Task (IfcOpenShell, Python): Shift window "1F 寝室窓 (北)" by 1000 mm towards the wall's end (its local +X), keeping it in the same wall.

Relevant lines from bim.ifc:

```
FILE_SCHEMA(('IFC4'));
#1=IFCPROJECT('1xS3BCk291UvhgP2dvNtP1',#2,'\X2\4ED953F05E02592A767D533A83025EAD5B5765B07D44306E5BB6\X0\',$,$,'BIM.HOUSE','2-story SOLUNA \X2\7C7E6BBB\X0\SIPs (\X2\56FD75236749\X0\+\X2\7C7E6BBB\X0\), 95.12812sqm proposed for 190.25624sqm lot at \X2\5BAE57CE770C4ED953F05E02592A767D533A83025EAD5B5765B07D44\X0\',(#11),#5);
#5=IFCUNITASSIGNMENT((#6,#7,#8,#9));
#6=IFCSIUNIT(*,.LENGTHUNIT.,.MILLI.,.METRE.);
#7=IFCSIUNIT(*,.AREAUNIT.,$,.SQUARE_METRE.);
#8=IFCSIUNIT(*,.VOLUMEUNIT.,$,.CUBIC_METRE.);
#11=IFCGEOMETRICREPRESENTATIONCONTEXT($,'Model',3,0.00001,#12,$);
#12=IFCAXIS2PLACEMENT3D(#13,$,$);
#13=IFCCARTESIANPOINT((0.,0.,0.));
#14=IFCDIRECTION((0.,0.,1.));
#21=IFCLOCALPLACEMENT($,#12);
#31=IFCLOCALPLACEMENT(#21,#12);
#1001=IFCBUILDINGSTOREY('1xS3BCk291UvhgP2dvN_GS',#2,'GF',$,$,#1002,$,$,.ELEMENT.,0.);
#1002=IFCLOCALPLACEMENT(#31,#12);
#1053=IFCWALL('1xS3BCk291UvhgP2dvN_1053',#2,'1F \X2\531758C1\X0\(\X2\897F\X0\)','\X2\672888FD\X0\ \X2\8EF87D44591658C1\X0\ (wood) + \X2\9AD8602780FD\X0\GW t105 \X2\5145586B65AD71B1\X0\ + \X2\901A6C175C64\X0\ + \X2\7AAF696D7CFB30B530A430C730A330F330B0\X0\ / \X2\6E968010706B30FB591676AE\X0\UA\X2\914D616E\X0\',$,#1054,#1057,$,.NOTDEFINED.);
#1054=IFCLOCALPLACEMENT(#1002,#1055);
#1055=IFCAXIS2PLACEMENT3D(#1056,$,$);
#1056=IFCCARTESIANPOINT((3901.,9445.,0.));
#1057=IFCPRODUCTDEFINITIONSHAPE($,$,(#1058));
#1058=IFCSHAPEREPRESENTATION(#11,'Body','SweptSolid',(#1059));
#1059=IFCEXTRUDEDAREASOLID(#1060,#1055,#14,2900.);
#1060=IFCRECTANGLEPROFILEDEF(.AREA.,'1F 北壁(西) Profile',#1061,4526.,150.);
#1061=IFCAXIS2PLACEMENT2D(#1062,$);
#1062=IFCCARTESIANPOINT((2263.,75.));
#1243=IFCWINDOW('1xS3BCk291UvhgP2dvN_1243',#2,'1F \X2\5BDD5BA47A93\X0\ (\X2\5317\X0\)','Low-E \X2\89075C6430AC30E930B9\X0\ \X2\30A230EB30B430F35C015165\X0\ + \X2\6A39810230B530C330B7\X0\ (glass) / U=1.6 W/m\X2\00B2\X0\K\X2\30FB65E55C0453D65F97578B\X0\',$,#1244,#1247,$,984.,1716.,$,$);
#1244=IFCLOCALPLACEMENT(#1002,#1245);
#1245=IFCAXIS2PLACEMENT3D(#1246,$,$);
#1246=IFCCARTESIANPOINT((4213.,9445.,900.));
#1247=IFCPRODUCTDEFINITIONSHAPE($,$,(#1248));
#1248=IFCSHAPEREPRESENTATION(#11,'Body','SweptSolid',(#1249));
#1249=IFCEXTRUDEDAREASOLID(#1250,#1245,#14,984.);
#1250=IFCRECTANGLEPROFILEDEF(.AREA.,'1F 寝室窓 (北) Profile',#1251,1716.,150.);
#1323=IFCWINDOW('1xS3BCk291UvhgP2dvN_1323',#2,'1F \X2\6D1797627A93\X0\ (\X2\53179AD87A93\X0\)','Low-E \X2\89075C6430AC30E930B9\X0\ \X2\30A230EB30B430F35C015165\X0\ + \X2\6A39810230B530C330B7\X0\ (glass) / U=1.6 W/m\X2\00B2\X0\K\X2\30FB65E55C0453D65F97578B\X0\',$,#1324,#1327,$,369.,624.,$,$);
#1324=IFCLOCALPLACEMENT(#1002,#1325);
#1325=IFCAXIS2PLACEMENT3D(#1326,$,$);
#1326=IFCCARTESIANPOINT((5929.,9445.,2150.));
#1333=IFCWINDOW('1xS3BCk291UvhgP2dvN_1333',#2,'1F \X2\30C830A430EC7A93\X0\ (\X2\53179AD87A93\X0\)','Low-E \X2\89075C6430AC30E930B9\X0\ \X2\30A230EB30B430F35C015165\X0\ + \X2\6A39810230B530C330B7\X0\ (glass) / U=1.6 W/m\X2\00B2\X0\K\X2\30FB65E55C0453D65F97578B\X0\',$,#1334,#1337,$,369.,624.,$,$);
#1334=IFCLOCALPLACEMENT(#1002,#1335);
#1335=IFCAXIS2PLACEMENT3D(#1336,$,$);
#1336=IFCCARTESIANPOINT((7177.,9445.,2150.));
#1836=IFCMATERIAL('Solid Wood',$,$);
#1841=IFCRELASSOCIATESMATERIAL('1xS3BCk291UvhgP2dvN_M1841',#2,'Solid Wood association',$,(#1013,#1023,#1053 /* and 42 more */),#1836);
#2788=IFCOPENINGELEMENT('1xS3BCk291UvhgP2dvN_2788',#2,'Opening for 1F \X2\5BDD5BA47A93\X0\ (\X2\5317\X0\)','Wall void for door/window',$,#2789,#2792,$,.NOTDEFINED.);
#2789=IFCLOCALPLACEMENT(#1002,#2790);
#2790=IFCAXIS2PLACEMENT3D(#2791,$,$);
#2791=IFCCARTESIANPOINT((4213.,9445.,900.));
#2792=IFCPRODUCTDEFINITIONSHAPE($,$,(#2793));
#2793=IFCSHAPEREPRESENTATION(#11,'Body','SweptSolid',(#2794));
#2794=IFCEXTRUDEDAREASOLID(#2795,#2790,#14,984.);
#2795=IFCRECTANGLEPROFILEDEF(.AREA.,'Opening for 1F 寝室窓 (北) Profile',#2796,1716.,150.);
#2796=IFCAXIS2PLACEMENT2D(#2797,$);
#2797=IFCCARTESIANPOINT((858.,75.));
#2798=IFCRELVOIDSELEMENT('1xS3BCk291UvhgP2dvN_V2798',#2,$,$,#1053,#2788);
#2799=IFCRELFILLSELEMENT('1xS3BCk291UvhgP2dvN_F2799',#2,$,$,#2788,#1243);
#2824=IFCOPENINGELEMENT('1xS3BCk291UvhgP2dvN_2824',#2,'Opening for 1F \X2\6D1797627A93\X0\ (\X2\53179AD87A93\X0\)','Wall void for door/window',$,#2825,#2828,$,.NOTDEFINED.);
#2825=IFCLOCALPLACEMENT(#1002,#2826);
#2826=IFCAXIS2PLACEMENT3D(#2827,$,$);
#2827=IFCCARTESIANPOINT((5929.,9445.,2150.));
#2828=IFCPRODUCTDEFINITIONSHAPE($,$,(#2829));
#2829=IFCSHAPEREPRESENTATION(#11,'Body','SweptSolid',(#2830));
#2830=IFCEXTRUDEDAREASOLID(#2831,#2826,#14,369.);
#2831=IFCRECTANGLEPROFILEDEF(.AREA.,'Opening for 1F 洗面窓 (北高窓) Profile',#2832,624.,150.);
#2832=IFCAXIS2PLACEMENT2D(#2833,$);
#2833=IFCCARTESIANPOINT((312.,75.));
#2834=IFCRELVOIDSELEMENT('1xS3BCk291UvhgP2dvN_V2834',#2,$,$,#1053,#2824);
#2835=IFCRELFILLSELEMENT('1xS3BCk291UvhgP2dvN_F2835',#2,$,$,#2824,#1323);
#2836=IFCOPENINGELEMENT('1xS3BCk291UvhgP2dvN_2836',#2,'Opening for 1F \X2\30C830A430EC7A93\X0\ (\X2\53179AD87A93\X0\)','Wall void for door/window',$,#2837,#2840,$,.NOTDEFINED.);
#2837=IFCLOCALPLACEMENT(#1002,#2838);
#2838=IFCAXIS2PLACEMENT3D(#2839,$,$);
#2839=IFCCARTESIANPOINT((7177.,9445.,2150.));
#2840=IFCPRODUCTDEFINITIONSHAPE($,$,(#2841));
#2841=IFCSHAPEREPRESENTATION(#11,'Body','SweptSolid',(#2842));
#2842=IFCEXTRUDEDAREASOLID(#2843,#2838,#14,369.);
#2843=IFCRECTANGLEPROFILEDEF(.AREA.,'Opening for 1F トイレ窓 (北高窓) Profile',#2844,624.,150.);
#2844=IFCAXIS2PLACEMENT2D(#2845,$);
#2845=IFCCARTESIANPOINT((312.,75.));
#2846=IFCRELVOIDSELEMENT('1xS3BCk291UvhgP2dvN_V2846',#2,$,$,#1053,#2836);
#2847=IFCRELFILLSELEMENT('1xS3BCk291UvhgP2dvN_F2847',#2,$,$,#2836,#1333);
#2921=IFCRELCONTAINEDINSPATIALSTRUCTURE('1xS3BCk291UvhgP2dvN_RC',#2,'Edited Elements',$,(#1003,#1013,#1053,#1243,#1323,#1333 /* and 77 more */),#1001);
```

```python
import ifcopenshell
import ifcopenshell.api.geometry
import ifcopenshell.util.placement
import ifcopenshell.util.unit

model = ifcopenshell.open("bim.ifc")
unit_scale = ifcopenshell.util.unit.calculate_unit_scale(model)

window = model.by_guid("1xS3BCk291UvhgP2dvN_1243")
opening = window.FillsVoids[0].RelatingOpeningElement
wall = opening.VoidsElements[0].RelatingBuildingElement

wall_matrix = ifcopenshell.util.placement.get_local_placement(wall.ObjectPlacement)
shift = wall_matrix[:3, 0] * 1 / unit_scale
before = ifcopenshell.util.placement.get_local_placement(window.ObjectPlacement)[:3, 3].copy()

# The window is not placed relative to its opening, so move both.
for product in (opening, window):
    matrix = ifcopenshell.util.placement.get_local_placement(product.ObjectPlacement)
    matrix[:3, 3] += shift
    ifcopenshell.api.geometry.edit_object_placement(model, product=product, matrix=matrix, is_si=False)

after = ifcopenshell.util.placement.get_local_placement(window.ObjectPlacement)[:3, 3]
print("window moved by", (after - before).round(3) + 0.0)

model.write("bim_edited.ifc")
```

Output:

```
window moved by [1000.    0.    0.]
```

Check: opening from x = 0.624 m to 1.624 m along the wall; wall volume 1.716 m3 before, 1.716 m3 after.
